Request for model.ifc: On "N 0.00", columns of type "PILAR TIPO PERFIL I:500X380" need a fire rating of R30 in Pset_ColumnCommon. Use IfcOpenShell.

First a look at what the model holds.

```python
import ifcopenshell
import ifcopenshell.util.element

model = ifcopenshell.open("model.ifc")
print(model.schema)
storey = next(s for s in model.by_type("IfcBuildingStorey") if s.Name == "N 0.00")
columns = [e for e in ifcopenshell.util.element.get_decomposition(storey) if e.is_a("IfcColumn")]
seen = {}
for e in columns:
    element_type = ifcopenshell.util.element.get_type(e)
    key = (element_type.Name if element_type != e and element_type else None, ifcopenshell.util.element.get_pset(e, "Pset_ColumnCommon", "FireRating"))
    seen[key] = seen.get(key, 0) + 1
for (name, value), count in sorted(seen.items(), key=str):
    print(count, "x", name, "|", value)
```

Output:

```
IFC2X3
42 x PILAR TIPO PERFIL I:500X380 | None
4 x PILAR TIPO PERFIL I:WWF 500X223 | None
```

```python
import ifcopenshell
import ifcopenshell.api.pset
import ifcopenshell.util.element

model = ifcopenshell.open("model.ifc")

storey = next(s for s in model.by_type("IfcBuildingStorey") if s.Name == "N 0.00")
columns = [e for e in ifcopenshell.util.element.get_decomposition(storey) if e.is_a("IfcColumn")]

count = 0
for e in columns:
    element_type = ifcopenshell.util.element.get_type(e)
    if element_type in (None, e) or element_type.Name != "PILAR TIPO PERFIL I:500X380":
        continue
    # add_pset returns the element's existing set when there is one.
    pset = ifcopenshell.api.pset.add_pset(model, product=e, name="Pset_ColumnCommon")
    ifcopenshell.api.pset.edit_pset(model, pset=pset, properties={"FireRating": "R30"})
    count += 1

print(count, "columns updated")

model.write("model-out.ifc")
```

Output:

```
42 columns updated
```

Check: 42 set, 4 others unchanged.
